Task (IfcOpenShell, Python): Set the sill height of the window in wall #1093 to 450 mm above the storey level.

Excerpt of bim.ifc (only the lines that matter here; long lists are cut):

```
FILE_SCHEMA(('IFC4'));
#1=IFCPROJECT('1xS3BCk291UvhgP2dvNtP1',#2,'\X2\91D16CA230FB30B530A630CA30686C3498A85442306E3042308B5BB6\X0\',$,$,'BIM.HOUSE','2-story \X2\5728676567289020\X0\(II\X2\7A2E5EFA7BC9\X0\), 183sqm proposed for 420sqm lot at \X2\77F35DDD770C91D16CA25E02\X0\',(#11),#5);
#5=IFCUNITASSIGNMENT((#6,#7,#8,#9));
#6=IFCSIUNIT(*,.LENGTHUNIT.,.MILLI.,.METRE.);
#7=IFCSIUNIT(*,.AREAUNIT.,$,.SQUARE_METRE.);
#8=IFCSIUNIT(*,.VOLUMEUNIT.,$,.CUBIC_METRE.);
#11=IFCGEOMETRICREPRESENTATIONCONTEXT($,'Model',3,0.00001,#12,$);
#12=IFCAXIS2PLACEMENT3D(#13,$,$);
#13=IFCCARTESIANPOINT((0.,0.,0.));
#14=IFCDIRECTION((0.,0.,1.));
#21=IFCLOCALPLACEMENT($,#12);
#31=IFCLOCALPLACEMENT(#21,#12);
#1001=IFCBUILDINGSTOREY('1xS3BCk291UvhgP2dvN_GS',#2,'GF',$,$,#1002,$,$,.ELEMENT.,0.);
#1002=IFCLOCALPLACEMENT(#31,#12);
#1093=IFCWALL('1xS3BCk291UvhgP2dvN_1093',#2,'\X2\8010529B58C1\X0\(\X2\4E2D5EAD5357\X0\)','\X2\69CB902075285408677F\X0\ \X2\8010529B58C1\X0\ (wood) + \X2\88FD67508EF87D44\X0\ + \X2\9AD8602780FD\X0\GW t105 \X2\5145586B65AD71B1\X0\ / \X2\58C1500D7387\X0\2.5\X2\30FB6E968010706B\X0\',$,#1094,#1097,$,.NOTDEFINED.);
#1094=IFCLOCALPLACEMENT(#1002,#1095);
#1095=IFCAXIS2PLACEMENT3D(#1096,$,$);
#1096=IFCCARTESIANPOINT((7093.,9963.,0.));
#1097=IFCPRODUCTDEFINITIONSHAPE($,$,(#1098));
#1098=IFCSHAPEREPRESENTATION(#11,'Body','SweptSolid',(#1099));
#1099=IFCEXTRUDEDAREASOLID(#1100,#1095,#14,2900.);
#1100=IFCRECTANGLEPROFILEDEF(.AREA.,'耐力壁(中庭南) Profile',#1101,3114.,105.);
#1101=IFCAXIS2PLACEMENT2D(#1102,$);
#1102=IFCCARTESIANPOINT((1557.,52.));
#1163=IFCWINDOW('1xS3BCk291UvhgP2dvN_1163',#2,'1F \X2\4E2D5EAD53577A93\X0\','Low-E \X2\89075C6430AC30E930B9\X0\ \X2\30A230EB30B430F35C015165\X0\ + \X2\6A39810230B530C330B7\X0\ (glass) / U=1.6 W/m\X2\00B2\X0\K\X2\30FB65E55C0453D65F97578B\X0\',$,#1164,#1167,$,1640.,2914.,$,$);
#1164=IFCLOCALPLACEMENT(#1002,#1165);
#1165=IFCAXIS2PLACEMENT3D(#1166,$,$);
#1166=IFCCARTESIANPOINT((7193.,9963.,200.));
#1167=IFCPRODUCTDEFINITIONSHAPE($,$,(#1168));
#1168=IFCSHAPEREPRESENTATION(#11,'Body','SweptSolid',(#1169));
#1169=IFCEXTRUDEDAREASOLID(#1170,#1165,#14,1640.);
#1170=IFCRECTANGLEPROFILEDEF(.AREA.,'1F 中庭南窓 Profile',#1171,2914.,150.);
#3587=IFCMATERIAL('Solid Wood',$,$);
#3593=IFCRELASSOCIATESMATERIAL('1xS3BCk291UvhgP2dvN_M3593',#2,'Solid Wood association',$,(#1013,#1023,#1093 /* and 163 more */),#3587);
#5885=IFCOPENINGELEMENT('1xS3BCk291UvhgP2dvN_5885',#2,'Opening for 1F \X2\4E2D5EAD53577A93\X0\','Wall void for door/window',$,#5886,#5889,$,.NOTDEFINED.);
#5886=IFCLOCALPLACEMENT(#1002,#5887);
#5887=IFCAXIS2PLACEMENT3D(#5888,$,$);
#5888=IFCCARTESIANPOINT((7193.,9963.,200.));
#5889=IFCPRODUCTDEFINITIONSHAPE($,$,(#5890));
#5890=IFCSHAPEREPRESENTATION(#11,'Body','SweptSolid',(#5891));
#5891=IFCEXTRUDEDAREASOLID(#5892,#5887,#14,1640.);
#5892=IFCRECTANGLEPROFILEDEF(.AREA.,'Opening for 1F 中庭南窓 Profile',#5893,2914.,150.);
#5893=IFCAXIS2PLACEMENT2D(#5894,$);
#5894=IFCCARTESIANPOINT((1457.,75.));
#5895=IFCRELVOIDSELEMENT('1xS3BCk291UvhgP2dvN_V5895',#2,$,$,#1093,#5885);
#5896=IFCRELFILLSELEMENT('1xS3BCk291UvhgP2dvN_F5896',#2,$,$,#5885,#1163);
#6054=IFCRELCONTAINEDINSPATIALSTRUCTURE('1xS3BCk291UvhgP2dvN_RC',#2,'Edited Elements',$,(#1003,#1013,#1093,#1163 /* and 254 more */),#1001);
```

```python
import numpy as np
import ifcopenshell
import ifcopenshell.api.geometry
import ifcopenshell.geom
import ifcopenshell.util.element
import ifcopenshell.util.placement
import ifcopenshell.util.shape
import ifcopenshell.util.unit

model = ifcopenshell.open("bim.ifc")
unit_scale = ifcopenshell.util.unit.calculate_unit_scale(model)

window = model.by_id(1163)
opening = window.FillsVoids[0].RelatingOpeningElement
storey = ifcopenshell.util.element.get_container(window, ifc_class="IfcBuildingStorey")
level = ifcopenshell.util.placement.get_local_placement(storey.ObjectPlacement)[2, 3]

# The opening's origin need not be at the sill, so measure its lowest point.
shape = ifcopenshell.geom.create_shape(ifcopenshell.geom.settings(), opening)
bottom = ifcopenshell.util.shape.get_shape_bottom_elevation(shape, shape.geometry) / unit_scale
dz = level + 0.45 / unit_scale - bottom

shift = np.array([0.0, 0.0, dz])
# The window is not placed relative to its opening, so move both.
for product in (opening, window):
    matrix = ifcopenshell.util.placement.get_local_placement(product.ObjectPlacement)
    matrix[:3, 3] += shift
    ifcopenshell.api.geometry.edit_object_placement(model, product=product, matrix=matrix, is_si=False)

print(f"moved by {dz * unit_scale:+.3f} m")

model.write("bim_edited.ifc")
```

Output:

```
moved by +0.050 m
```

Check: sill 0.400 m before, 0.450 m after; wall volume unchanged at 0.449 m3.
